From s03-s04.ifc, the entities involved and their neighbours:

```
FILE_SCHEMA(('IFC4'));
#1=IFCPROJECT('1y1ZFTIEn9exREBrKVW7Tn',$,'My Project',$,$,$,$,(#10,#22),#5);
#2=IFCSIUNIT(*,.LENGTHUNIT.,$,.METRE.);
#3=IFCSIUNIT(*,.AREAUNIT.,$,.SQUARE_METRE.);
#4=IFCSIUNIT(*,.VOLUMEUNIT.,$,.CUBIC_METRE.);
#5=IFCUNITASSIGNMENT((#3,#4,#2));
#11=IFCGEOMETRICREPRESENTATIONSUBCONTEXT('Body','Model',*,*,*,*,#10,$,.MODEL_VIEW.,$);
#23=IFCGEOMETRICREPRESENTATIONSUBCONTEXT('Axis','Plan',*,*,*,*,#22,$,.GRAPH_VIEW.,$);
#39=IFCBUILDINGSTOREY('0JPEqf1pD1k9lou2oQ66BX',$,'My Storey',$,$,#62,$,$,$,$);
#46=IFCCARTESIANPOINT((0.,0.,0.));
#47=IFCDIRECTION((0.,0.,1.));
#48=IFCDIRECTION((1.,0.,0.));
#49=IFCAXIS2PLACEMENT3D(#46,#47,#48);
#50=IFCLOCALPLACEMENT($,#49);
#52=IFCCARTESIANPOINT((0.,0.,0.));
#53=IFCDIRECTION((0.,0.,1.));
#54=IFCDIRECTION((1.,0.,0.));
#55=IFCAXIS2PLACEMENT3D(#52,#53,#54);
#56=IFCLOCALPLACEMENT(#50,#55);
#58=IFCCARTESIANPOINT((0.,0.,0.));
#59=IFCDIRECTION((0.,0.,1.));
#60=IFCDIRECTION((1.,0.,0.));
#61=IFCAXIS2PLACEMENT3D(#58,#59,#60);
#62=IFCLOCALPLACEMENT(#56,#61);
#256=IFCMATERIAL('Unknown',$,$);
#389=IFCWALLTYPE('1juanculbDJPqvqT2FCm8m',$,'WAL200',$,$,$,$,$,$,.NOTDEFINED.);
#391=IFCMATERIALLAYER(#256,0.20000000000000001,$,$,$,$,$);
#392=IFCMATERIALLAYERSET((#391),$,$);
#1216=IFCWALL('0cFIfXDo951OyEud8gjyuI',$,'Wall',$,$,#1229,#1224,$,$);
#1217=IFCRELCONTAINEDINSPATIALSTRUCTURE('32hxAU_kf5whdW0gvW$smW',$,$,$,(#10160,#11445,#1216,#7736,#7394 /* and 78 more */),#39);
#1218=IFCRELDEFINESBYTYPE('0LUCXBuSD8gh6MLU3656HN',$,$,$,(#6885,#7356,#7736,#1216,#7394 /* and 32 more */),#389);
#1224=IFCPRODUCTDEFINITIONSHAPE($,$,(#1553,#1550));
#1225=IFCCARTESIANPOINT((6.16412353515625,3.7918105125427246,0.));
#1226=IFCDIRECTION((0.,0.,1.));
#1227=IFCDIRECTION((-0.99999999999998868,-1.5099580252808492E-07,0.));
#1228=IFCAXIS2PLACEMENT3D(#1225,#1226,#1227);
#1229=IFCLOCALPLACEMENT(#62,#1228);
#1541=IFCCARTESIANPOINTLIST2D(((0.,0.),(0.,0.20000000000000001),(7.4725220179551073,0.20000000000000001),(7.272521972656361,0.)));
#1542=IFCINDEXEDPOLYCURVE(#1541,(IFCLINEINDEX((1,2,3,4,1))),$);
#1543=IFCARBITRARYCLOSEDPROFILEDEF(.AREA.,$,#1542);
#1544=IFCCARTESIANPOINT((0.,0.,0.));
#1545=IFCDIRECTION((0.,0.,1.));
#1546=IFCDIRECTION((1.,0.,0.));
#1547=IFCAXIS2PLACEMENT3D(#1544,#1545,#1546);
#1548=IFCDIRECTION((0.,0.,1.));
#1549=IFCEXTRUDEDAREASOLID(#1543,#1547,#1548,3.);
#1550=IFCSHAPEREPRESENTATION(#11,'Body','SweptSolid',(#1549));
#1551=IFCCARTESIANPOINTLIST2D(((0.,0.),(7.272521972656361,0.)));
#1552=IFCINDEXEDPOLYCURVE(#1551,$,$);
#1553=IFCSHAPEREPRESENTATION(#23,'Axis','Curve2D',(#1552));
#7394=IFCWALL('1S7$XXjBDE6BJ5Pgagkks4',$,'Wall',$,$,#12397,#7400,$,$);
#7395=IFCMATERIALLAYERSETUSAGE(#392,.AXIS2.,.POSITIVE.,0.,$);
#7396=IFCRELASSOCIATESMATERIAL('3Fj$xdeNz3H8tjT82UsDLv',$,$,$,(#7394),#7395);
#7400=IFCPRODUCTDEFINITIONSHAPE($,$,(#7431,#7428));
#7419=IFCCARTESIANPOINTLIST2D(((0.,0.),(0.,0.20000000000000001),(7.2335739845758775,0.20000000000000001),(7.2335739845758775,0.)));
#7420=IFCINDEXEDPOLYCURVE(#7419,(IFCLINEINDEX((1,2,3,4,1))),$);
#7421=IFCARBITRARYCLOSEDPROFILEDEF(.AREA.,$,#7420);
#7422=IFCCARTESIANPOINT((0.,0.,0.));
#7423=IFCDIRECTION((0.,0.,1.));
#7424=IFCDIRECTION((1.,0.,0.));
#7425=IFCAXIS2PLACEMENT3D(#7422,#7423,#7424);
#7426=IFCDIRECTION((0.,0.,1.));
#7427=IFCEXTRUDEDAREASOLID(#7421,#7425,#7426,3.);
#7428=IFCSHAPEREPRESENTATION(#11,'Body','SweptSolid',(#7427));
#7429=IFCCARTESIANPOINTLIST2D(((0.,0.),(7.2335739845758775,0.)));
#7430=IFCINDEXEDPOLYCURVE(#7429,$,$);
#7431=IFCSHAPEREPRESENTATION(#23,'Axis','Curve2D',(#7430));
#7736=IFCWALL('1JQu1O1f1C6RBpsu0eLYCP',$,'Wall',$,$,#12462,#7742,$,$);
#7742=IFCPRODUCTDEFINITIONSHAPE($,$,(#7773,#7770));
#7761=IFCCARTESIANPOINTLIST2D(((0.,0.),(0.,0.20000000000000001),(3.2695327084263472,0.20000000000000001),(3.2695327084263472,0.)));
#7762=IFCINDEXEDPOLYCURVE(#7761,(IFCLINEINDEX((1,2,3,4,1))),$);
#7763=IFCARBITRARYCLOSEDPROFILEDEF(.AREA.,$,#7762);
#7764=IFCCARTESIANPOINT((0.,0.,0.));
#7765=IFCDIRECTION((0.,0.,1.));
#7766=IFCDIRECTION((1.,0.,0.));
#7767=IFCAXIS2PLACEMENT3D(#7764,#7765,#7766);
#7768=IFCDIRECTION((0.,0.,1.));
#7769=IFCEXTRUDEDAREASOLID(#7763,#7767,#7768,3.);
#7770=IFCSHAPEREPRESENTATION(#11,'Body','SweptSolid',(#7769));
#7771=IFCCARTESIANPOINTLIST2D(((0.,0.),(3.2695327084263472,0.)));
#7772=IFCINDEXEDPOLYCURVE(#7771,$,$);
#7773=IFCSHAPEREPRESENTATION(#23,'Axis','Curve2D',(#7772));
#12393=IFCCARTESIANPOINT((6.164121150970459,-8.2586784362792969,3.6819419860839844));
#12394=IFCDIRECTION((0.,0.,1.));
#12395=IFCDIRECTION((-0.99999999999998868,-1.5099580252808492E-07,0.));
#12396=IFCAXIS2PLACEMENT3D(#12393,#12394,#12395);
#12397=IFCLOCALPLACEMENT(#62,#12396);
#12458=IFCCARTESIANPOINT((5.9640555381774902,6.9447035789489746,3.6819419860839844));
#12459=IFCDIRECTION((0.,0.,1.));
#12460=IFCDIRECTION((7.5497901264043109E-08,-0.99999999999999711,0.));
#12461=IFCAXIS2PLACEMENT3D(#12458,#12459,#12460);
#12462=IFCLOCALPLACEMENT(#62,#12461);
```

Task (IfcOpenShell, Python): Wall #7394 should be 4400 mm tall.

```python
import ifcopenshell
import ifcopenshell.geom
import ifcopenshell.util.representation
import ifcopenshell.util.shape
import ifcopenshell.util.unit

model = ifcopenshell.open("s03-s04.ifc")
unit_scale = ifcopenshell.util.unit.calculate_unit_scale(model)
settings = ifcopenshell.geom.settings()


def volume(element):
    """Net volume in cubic metres, openings subtracted."""
    shape = ifcopenshell.geom.create_shape(settings, element)
    return ifcopenshell.util.shape.get_volume(shape.geometry)


wall = model.by_guid("1S7$XXjBDE6BJ5Pgagkks4")
before = volume(wall)

body = ifcopenshell.util.representation.get_representation(wall, "Model", "Body")
solid = body.Items[0]
old_height = solid.Depth
solid.Depth = 4.4 / unit_scale
after = volume(wall)

print(f"height {old_height:g} -> {solid.Depth:g}, volume {before:.3f} -> {after:.3f} m3")

model.write("s03-s04-out.ifc")
```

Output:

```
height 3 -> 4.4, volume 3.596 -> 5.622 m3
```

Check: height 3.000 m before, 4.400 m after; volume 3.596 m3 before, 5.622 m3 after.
